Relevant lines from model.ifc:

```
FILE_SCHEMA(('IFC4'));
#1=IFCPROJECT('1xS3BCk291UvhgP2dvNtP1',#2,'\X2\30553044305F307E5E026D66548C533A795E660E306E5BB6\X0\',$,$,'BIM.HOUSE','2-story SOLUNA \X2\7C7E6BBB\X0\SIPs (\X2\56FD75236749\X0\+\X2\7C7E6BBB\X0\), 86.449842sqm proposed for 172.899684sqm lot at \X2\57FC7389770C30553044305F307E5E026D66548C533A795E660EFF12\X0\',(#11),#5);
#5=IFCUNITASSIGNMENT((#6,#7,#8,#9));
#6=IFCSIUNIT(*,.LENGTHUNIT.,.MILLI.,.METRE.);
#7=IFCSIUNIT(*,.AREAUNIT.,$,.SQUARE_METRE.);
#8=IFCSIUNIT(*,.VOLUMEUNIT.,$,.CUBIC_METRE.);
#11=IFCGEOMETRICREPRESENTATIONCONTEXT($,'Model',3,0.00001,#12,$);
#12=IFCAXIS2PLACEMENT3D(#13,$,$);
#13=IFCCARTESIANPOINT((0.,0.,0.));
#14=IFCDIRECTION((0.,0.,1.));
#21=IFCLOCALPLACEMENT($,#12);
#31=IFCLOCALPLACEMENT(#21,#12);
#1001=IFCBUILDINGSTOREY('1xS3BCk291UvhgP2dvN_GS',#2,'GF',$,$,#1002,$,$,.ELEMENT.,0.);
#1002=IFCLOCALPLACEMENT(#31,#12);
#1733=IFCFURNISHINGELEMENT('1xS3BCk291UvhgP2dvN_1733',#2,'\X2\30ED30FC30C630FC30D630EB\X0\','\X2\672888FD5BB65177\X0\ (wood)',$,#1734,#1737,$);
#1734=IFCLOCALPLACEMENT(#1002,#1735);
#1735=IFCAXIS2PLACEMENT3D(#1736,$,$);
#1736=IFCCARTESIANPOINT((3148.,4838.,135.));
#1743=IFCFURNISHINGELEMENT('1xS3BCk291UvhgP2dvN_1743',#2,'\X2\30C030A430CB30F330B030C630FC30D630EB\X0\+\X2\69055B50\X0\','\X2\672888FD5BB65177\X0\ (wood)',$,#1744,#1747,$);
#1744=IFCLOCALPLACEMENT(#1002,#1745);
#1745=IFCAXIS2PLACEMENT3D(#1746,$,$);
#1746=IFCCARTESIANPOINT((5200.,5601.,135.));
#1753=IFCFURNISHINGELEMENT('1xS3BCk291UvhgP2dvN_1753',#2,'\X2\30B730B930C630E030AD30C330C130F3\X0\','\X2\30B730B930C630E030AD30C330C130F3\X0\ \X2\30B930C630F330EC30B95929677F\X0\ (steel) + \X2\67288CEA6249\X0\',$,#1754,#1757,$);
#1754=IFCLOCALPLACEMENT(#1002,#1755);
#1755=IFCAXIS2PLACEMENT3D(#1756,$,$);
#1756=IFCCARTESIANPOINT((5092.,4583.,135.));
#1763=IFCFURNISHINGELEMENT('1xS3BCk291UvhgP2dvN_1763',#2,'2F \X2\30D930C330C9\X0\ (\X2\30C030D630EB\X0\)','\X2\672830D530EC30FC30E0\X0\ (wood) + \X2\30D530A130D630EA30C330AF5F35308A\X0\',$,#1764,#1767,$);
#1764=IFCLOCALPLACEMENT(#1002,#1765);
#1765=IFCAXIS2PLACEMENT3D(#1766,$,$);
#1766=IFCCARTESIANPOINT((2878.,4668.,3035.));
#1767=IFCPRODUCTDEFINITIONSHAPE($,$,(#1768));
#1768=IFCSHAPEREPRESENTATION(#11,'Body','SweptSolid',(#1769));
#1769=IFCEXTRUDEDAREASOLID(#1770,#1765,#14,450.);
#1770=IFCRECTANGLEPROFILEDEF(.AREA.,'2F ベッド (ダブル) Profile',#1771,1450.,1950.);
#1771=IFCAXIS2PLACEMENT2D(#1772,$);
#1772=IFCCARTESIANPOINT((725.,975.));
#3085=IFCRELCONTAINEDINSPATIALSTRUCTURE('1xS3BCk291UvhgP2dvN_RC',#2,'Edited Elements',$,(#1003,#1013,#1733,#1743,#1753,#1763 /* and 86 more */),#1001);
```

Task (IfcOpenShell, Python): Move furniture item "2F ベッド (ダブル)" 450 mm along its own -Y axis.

```python
import ifcopenshell
import ifcopenshell.api.geometry
import ifcopenshell.util.placement

model = ifcopenshell.open("model.ifc")

item = model.by_guid("1xS3BCk291UvhgP2dvN_1763")
matrix = ifcopenshell.util.placement.get_local_placement(item.ObjectPlacement)
matrix[:3, 3] -= matrix[:3, 1] * 450.0
ifcopenshell.api.geometry.edit_object_placement(model, product=item, matrix=matrix, is_si=False)

print(ifcopenshell.util.placement.get_local_placement(item.ObjectPlacement).round(3) + 0.0)

model.write("model-out.ifc")
```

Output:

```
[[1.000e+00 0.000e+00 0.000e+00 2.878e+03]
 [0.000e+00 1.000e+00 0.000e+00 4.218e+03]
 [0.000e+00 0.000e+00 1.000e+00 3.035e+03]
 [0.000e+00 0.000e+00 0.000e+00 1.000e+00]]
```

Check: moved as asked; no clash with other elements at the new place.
